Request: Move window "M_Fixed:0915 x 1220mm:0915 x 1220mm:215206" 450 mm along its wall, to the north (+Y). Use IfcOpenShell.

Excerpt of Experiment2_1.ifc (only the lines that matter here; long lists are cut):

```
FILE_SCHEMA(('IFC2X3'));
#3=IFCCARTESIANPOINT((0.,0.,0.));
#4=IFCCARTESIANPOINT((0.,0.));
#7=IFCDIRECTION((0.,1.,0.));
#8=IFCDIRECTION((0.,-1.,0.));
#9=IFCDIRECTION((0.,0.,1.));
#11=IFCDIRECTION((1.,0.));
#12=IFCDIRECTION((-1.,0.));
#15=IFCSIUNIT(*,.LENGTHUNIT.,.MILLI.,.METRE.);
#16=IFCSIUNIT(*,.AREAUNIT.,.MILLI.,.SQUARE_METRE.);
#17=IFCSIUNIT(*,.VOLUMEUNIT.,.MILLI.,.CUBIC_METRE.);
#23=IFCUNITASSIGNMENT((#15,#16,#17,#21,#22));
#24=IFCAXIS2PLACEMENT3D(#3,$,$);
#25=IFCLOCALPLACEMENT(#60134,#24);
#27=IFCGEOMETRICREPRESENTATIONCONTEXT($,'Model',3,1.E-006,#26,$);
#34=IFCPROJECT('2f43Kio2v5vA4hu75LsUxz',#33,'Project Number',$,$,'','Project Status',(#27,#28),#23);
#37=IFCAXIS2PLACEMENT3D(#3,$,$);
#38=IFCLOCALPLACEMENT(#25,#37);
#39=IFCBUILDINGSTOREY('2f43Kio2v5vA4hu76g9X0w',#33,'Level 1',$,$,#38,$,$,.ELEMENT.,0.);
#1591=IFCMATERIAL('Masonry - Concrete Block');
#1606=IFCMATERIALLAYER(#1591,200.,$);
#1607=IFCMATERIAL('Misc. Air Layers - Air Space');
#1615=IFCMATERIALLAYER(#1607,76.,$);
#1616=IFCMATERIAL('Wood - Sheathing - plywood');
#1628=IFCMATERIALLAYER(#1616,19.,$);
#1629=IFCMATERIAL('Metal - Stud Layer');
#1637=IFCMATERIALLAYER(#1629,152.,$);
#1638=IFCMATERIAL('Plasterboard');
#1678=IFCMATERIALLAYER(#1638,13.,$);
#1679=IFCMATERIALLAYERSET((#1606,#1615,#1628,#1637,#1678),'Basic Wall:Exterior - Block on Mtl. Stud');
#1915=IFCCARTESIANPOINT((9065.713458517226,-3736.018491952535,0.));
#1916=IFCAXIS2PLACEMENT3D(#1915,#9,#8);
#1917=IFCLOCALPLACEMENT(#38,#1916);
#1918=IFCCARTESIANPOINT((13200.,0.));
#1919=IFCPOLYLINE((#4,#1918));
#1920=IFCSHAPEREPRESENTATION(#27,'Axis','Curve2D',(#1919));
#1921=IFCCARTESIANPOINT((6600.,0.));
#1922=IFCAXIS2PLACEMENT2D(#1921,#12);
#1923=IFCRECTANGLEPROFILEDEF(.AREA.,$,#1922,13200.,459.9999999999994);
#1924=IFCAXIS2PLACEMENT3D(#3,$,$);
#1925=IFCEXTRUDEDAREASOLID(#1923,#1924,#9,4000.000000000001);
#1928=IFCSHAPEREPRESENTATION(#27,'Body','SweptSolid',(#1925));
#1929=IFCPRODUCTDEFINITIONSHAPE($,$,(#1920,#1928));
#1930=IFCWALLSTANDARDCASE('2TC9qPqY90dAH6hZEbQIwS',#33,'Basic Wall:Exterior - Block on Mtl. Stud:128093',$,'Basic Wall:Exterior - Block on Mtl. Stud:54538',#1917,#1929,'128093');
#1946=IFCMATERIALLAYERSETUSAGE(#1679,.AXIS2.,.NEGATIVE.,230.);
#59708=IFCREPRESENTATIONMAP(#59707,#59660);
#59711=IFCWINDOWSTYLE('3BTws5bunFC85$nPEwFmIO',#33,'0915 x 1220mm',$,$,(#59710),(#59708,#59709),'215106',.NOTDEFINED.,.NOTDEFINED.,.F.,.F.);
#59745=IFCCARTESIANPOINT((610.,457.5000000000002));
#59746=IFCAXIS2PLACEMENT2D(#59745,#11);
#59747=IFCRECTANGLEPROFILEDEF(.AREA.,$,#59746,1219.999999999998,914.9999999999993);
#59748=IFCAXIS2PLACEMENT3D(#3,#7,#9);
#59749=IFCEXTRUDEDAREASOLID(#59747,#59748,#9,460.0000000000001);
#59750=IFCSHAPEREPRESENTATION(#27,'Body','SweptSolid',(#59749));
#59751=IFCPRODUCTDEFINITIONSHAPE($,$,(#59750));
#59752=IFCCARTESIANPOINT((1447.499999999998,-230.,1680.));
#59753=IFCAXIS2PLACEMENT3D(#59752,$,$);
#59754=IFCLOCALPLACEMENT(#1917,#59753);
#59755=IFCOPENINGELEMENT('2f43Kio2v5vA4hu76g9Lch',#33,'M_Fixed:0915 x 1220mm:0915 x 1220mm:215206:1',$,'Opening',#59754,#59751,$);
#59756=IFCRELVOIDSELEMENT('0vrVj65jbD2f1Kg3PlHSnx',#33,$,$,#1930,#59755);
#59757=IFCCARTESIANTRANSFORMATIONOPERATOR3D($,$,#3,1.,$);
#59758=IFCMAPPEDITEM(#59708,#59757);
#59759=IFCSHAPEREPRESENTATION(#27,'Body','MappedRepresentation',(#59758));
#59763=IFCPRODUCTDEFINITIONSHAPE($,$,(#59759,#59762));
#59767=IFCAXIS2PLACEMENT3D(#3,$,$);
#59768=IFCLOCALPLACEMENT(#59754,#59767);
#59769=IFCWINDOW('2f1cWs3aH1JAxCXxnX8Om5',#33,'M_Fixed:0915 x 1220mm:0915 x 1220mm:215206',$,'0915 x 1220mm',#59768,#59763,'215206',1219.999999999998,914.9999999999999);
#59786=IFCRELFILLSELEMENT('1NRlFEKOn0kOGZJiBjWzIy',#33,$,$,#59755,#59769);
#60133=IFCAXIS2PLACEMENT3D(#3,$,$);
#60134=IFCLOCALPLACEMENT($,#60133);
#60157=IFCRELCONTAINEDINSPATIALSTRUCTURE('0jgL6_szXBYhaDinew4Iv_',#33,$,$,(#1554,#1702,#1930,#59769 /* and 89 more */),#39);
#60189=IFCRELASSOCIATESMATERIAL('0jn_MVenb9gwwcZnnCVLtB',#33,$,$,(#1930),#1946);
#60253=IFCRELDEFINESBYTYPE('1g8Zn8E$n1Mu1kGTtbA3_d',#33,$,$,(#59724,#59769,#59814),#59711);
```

```python
import ifcopenshell
import ifcopenshell.api.geometry
import ifcopenshell.util.placement
import ifcopenshell.util.unit

model = ifcopenshell.open("Experiment2_1.ifc")
unit_scale = ifcopenshell.util.unit.calculate_unit_scale(model)

window = model.by_guid("2f1cWs3aH1JAxCXxnX8Om5")
opening = window.FillsVoids[0].RelatingOpeningElement
wall = opening.VoidsElements[0].RelatingBuildingElement

wall_matrix = ifcopenshell.util.placement.get_local_placement(wall.ObjectPlacement)
shift = wall_matrix[:3, 0] * -0.45 / unit_scale
before = ifcopenshell.util.placement.get_local_placement(window.ObjectPlacement)[:3, 3].copy()

# The window is placed relative to its opening, so it follows when the opening moves.
matrix = ifcopenshell.util.placement.get_local_placement(opening.ObjectPlacement)
matrix[:3, 3] += shift
ifcopenshell.api.geometry.edit_object_placement(
    model, product=opening, matrix=matrix, is_si=False, should_transform_children=True
)

after = ifcopenshell.util.placement.get_local_placement(window.ObjectPlacement)[:3, 3]
print("window moved by", (after - before).round(3) + 0.0)

model.write("Experiment2_1-out.ifc")
```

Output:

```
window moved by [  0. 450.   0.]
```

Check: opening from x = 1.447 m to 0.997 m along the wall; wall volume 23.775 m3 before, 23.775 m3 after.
